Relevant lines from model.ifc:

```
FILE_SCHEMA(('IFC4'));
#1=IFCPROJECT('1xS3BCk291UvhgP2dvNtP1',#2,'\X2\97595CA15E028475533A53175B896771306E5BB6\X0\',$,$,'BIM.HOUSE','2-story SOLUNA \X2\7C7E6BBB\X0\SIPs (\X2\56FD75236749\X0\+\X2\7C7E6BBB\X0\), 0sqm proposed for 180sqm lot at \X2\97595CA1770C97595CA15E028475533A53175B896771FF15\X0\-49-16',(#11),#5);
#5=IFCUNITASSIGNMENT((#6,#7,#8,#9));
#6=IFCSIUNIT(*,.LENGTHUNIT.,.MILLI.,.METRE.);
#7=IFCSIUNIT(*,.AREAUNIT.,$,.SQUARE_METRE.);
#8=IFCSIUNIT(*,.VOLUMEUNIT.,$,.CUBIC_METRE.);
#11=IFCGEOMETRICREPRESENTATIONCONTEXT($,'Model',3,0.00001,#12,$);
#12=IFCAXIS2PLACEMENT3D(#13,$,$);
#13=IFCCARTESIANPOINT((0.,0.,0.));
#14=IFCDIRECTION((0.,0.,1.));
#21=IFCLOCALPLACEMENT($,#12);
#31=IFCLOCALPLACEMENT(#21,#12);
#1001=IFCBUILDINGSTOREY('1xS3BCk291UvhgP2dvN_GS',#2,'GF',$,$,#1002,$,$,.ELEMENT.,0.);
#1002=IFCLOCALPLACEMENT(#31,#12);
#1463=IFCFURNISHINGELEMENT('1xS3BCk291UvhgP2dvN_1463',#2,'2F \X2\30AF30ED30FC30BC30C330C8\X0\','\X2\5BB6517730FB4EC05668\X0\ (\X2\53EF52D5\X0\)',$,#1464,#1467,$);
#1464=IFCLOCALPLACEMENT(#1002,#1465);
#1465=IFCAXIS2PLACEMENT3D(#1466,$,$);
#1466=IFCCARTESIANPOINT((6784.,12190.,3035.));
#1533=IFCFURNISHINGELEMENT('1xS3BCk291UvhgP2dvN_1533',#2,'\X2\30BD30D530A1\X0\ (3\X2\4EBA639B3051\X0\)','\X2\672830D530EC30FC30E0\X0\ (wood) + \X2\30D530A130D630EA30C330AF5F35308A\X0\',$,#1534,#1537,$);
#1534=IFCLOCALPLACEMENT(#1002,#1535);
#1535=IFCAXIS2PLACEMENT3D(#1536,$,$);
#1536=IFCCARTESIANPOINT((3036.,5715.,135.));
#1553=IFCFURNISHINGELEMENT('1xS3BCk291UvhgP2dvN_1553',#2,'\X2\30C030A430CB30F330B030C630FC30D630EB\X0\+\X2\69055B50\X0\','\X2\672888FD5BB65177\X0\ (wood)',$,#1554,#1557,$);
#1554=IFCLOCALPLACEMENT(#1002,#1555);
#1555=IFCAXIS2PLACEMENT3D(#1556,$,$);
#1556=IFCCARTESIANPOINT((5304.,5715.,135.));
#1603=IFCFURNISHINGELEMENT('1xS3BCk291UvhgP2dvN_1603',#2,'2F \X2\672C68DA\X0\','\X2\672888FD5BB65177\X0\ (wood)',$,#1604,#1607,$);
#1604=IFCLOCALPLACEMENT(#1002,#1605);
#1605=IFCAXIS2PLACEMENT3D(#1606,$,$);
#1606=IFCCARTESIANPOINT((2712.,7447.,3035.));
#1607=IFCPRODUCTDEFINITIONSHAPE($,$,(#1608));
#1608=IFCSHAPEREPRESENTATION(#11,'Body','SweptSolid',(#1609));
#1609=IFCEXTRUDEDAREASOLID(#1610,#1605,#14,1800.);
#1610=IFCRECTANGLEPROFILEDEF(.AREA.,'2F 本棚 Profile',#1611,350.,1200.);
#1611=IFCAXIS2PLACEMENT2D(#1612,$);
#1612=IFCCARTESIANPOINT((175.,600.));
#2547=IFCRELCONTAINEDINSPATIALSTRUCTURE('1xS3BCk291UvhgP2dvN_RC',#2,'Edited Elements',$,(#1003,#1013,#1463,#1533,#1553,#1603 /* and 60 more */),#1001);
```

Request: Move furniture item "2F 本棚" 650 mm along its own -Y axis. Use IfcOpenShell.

```python
import ifcopenshell
import ifcopenshell.api.geometry
import ifcopenshell.util.placement

model = ifcopenshell.open("model.ifc")

item = model.by_id(1603)
matrix = ifcopenshell.util.placement.get_local_placement(item.ObjectPlacement)
matrix[:3, 3] -= matrix[:3, 1] * 650.0
ifcopenshell.api.geometry.edit_object_placement(model, product=item, matrix=matrix, is_si=False)

print(ifcopenshell.util.placement.get_local_placement(item.ObjectPlacement).round(3) + 0.0)

model.write("model-out.ifc")
```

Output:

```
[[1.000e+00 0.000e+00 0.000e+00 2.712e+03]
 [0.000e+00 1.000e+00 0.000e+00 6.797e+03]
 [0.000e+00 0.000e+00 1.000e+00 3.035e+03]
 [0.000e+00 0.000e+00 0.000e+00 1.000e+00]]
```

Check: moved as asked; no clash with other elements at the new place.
